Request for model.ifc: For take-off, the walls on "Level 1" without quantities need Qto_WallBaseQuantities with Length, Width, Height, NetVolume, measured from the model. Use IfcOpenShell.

First a look at what the model holds.

```python
import ifcopenshell
import ifcopenshell.util.element
import ifcopenshell.util.unit

model = ifcopenshell.open("model.ifc")
print(model.schema)
for unit_type in ("LENGTHUNIT", "AREAUNIT", "VOLUMEUNIT"):
    print(unit_type, ifcopenshell.util.unit.calculate_unit_scale(model, unit_type))
storey = next(s for s in model.by_type("IfcBuildingStorey") if s.Name == "Level 1")
walls = [e for e in ifcopenshell.util.element.get_decomposition(storey) if e.is_a("IfcWall")]
for e in sorted(walls, key=lambda e: e.id()):
    print(e.id(), e.is_a(), e.Name, list(ifcopenshell.util.element.get_psets(e, qtos_only=True)), sep=" | ")
```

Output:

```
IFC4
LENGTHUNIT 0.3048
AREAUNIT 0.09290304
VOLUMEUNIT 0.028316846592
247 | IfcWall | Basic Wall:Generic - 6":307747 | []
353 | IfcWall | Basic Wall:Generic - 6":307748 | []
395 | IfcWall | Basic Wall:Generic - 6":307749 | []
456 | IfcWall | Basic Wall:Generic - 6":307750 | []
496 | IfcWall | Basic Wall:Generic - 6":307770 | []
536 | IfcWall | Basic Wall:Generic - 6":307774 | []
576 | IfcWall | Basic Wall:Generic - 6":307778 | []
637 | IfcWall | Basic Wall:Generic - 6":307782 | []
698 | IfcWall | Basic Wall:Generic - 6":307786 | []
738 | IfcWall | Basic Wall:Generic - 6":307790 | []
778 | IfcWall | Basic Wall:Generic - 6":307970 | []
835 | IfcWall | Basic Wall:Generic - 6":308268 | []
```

```python
import ifcopenshell
import ifcopenshell.api.pset
import ifcopenshell.geom
import ifcopenshell.util.element
import ifcopenshell.util.shape
import ifcopenshell.util.unit

model = ifcopenshell.open("model.ifc")
unit_scale = ifcopenshell.util.unit.calculate_unit_scale(model)
volume_scale = ifcopenshell.util.unit.calculate_unit_scale(model, "VOLUMEUNIT")
settings = ifcopenshell.geom.settings()

storey = next(s for s in model.by_type("IfcBuildingStorey") if s.Name == "Level 1")
walls = [e for e in ifcopenshell.util.element.get_decomposition(storey) if e.is_a("IfcWall")]

for e in sorted(walls, key=lambda e: e.id()):
    if ifcopenshell.util.element.get_psets(e, qtos_only=True, should_inherit=False):
        continue
    # Geometry comes back in metres, in the element's own axes.
    shape = ifcopenshell.geom.create_shape(settings, e)
    values = {
        "Length": ifcopenshell.util.shape.get_x(shape.geometry) / unit_scale,
        "Width": ifcopenshell.util.shape.get_y(shape.geometry) / unit_scale,
        "Height": ifcopenshell.util.shape.get_z(shape.geometry) / unit_scale,
        "NetVolume": ifcopenshell.util.shape.get_volume(shape.geometry) / volume_scale,
    }
    qto = ifcopenshell.api.pset.add_qto(model, product=e, name="Qto_WallBaseQuantities")
    ifcopenshell.api.pset.edit_qto(model, qto=qto, properties=values)
    print(e.id(), {k: round(v, 3) for k, v in values.items()})

model.write("model_v2.ifc")
```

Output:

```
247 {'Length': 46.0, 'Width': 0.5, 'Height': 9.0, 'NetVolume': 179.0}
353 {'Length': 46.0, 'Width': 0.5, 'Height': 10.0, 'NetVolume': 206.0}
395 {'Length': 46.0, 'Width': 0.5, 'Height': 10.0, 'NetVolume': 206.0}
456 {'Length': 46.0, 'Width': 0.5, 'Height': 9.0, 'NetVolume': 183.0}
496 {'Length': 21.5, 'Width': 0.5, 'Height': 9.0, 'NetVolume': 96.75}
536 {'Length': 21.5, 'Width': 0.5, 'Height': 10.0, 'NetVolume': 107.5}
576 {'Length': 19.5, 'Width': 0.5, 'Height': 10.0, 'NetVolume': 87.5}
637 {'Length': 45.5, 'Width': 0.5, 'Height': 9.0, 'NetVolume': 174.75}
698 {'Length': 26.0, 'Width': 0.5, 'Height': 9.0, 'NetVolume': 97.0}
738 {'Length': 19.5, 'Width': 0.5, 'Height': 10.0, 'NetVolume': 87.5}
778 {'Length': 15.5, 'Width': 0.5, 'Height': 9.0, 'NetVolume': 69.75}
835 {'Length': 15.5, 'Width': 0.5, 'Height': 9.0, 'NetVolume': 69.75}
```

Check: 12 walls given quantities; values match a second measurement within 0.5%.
